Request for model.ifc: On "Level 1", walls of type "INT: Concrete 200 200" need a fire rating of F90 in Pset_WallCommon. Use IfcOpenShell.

First a look at what the model holds.

```python
import ifcopenshell
import ifcopenshell.util.element

model = ifcopenshell.open("model.ifc")
print(model.schema)
storey = next(s for s in model.by_type("IfcBuildingStorey") if s.Name == "Level 1")
walls = [e for e in ifcopenshell.util.element.get_decomposition(storey) if e.is_a("IfcWall")]
seen = {}
for e in walls:
    element_type = ifcopenshell.util.element.get_type(e)
    key = (element_type.Name if element_type != e and element_type else None, ifcopenshell.util.element.get_pset(e, "Pset_WallCommon", "FireRating"))
    seen[key] = seen.get(key, 0) + 1
for (name, value), count in sorted(seen.items(), key=str):
    print(count, "x", name, "|", value)
```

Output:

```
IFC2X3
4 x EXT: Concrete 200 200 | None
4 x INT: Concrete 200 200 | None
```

```python
import ifcopenshell
import ifcopenshell.api.pset
import ifcopenshell.util.element

model = ifcopenshell.open("model.ifc")

storey = next(s for s in model.by_type("IfcBuildingStorey") if s.Name == "Level 1")
walls = [e for e in ifcopenshell.util.element.get_decomposition(storey) if e.is_a("IfcWall")]

count = 0
for e in walls:
    element_type = ifcopenshell.util.element.get_type(e)
    if element_type in (None, e) or element_type.Name != "INT: Concrete 200 200":
        continue
    # add_pset returns the element's existing set when there is one.
    pset = ifcopenshell.api.pset.add_pset(model, product=e, name="Pset_WallCommon")
    ifcopenshell.api.pset.edit_pset(model, pset=pset, properties={"FireRating": "F90"})
    count += 1

print(count, "walls updated")

model.write("model_v2.ifc")
```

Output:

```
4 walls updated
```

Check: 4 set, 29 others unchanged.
